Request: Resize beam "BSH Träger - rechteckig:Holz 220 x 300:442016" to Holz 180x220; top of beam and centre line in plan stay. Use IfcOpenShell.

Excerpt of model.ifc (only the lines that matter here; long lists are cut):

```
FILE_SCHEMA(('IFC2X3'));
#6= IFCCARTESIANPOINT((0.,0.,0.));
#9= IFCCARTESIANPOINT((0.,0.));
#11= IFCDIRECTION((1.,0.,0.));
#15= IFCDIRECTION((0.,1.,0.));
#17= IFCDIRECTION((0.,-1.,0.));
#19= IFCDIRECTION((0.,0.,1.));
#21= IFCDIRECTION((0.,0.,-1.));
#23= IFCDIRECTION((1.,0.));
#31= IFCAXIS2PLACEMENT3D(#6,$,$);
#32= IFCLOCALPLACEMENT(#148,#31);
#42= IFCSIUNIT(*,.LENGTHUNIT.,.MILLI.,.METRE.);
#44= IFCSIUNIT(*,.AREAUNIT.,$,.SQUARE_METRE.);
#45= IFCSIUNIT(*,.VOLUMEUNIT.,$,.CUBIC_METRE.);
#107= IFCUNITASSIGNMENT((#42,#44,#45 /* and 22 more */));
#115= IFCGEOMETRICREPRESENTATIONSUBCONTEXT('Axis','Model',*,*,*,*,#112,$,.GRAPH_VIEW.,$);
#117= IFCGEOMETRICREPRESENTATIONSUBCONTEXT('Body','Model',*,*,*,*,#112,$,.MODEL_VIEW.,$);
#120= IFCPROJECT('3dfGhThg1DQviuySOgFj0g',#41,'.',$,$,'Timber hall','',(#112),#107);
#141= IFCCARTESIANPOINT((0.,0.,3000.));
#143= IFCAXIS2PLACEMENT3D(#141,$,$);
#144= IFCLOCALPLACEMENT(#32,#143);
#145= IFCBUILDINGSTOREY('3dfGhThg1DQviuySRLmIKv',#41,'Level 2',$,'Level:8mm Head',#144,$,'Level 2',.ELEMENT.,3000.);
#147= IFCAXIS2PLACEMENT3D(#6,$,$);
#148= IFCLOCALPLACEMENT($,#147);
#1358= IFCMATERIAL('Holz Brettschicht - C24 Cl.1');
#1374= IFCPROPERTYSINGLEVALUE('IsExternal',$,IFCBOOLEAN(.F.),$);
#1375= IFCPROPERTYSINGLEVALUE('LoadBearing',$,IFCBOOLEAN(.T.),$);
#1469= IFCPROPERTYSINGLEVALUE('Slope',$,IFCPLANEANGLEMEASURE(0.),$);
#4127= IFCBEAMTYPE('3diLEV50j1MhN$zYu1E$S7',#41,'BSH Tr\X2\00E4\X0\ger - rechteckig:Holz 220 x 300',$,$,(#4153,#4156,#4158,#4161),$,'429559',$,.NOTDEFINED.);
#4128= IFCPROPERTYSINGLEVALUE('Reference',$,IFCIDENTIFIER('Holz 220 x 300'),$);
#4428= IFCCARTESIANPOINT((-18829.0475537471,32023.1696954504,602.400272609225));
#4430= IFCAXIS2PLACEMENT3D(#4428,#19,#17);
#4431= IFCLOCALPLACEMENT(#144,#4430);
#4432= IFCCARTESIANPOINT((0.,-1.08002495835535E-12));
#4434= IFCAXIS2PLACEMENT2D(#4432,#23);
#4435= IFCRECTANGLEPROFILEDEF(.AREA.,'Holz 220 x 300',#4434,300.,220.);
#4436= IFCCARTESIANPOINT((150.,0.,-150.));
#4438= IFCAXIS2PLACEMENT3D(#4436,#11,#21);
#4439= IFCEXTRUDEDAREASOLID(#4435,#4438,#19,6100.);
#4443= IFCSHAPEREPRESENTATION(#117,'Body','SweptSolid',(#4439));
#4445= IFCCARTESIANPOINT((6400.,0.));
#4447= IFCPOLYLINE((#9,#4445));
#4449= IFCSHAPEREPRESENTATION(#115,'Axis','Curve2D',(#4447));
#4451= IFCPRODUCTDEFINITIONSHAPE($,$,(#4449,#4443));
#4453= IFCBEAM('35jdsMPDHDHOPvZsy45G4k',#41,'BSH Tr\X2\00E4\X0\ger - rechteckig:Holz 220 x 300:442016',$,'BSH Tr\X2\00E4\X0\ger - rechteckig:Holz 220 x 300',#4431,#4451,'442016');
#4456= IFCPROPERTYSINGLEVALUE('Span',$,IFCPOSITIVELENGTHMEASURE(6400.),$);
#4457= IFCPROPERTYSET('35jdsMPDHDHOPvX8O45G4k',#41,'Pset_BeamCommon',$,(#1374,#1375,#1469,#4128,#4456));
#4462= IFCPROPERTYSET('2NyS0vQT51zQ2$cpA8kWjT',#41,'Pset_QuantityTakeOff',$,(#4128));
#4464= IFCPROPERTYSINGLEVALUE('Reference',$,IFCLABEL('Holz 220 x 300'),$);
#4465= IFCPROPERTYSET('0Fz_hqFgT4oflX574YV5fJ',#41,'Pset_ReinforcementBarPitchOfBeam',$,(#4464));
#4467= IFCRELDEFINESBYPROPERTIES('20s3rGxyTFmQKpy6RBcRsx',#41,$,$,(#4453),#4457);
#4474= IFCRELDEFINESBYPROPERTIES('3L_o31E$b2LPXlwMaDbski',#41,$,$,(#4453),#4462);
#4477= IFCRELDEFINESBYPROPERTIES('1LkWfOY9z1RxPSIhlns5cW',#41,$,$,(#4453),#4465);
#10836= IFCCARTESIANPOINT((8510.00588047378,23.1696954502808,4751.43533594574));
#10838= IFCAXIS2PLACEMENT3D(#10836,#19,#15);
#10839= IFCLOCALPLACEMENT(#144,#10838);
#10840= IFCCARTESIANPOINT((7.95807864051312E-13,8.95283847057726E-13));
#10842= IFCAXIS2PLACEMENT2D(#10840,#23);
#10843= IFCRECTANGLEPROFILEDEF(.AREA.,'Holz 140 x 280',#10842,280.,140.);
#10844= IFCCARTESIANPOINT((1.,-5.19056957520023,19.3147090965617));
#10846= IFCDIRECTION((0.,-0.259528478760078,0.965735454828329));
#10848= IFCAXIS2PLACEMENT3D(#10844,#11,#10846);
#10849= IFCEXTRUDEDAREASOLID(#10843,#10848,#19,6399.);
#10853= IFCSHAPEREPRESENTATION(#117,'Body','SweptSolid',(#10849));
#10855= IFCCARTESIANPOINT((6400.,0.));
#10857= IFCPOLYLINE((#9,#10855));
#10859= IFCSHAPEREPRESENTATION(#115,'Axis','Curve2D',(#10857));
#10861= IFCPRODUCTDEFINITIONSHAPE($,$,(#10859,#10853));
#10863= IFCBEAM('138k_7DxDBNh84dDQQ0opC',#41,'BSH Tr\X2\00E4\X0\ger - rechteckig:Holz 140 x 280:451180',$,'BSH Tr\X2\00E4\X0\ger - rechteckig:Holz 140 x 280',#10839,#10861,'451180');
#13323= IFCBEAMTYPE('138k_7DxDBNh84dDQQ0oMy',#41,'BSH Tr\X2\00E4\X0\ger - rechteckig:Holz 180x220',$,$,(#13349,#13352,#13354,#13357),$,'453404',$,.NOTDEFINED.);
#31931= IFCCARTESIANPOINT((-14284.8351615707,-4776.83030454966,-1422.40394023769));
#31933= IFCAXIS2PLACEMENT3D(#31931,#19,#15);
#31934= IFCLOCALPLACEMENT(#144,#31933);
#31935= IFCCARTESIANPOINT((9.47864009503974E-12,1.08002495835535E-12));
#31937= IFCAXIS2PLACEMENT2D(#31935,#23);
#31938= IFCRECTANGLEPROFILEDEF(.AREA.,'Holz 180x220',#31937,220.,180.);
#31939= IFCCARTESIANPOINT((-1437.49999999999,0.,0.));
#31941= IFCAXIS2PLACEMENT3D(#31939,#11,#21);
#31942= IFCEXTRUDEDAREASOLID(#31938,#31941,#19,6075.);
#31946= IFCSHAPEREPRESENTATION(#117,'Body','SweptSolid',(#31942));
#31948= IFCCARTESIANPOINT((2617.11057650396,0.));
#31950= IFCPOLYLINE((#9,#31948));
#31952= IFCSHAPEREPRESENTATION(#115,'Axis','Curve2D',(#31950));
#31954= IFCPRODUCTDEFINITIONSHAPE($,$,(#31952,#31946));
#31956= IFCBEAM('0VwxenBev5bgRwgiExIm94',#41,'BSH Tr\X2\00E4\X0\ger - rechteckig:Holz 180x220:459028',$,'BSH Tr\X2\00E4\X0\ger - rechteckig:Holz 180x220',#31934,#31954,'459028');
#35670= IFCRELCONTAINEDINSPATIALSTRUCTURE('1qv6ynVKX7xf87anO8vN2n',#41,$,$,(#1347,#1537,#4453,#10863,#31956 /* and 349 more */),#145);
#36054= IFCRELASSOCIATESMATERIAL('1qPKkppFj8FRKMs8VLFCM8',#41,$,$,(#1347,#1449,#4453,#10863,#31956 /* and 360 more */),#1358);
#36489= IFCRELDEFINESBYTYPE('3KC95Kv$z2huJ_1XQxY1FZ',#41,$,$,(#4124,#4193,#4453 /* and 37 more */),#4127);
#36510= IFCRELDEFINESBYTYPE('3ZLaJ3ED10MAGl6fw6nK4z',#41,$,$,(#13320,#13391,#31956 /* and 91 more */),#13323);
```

```python
import ifcopenshell
import ifcopenshell.api.pset
import ifcopenshell.api.type
import ifcopenshell.util.element
import ifcopenshell.util.representation

model = ifcopenshell.open("model.ifc")

member = model.by_id(4453)
source = next(p for p in model.by_type("IfcRectangleProfileDef") if p.ProfileName == "Holz 180x220")

body = ifcopenshell.util.representation.get_representation(member, "Model", "Body")
solid = body.Items[0]
old_profile = solid.SweptArea

# Copy the section's sizes but keep this member's own profile position.
profile = ifcopenshell.util.element.copy(model, source)
# Profiles are centred, so shift by half the change in depth to hold the top.
shift = (old_profile.XDim - profile.XDim) / 2
x, y = old_profile.Position.Location.Coordinates
up = (-1.0, 0.0)  # upwards, in the solid's own plane
location = model.createIfcCartesianPoint((x + up[0] * shift, y + up[1] * shift))
profile.Position = model.createIfcAxis2Placement2D(location, old_profile.Position.RefDirection)
solid.SweptArea = profile
if not model.get_total_inverses(old_profile):
    ifcopenshell.util.element.remove_deep2(model, old_profile)

new_type = model.by_guid("138k_7DxDBNh84dDQQ0oMy")
ifcopenshell.api.type.assign_type(
    model, related_objects=[member], relating_type=new_type, should_map_representations=False
)
member.Name = member.Name.replace("Holz 220 x 300", "Holz 180x220")
member.ObjectType = "BSH Träger - rechteckig:Holz 180x220"
pset = model.by_id(ifcopenshell.util.element.get_pset(member, "Pset_BeamCommon", should_inherit=False)["id"])
ifcopenshell.api.pset.edit_pset(model, pset=pset, properties={"Reference": "Holz 180x220"})
pset = model.by_id(ifcopenshell.util.element.get_pset(member, "Pset_QuantityTakeOff", should_inherit=False)["id"])
ifcopenshell.api.pset.edit_pset(model, pset=pset, properties={"Reference": "Holz 180x220"})
pset = model.by_id(ifcopenshell.util.element.get_pset(member, "Pset_ReinforcementBarPitchOfBeam", should_inherit=False)["id"])
ifcopenshell.api.pset.edit_pset(model, pset=pset, properties={"Reference": "Holz 180x220"})

print(solid.SweptArea)

model.write("model_rev.ifc")
```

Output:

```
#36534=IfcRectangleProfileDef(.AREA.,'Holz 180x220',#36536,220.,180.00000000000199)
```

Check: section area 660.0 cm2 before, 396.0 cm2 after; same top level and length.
